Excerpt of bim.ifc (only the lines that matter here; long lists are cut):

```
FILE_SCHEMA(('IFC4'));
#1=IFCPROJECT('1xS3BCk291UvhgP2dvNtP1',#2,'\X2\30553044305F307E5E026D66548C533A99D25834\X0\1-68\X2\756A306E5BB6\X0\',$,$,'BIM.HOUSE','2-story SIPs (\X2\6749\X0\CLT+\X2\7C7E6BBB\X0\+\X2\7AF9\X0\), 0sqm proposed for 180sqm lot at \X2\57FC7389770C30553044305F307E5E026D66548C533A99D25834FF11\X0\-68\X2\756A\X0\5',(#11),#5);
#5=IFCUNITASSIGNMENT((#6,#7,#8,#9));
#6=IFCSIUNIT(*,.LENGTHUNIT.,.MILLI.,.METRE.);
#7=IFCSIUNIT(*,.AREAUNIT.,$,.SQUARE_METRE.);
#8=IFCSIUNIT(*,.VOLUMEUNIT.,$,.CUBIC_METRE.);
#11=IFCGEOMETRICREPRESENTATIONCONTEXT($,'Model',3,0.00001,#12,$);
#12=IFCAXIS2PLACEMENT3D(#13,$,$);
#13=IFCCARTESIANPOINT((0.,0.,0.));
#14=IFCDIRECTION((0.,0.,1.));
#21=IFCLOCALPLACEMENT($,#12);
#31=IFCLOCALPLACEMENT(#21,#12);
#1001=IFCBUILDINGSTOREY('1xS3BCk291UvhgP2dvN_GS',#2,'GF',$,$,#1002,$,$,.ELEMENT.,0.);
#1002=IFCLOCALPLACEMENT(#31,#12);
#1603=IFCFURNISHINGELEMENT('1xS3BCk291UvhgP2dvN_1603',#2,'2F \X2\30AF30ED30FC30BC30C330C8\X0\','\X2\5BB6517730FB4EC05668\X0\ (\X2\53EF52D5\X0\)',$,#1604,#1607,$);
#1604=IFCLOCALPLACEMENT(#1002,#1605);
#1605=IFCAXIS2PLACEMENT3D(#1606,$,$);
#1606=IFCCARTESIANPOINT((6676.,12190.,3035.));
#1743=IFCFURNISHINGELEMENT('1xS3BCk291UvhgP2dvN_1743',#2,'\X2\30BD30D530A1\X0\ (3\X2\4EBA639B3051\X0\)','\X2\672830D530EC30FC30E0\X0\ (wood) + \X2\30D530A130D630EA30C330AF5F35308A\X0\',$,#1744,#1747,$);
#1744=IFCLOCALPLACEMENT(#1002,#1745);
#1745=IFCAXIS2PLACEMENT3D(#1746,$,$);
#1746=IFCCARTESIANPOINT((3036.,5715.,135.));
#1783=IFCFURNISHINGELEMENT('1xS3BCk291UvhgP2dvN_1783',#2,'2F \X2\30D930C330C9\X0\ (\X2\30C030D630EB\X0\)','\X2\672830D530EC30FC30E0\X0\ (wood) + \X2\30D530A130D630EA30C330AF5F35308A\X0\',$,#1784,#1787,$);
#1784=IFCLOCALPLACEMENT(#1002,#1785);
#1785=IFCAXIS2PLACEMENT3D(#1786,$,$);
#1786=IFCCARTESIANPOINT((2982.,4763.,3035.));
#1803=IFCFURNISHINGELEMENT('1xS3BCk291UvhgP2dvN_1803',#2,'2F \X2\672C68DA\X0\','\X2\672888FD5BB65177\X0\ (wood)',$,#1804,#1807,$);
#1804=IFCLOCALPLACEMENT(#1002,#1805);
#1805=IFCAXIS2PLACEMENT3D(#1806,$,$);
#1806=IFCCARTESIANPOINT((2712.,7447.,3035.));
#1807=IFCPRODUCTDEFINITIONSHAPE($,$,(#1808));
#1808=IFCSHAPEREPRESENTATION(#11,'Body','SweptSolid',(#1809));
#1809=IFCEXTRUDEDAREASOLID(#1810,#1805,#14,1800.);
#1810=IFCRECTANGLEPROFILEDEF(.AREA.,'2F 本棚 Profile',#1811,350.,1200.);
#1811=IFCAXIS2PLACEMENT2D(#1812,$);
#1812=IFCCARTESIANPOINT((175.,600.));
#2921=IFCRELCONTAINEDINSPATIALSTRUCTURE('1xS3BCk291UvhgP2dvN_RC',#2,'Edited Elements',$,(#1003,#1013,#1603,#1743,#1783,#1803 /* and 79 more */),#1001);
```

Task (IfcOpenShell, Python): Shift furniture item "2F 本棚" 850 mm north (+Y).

```python
import ifcopenshell
import ifcopenshell.api.geometry
import ifcopenshell.util.placement
import ifcopenshell.util.unit

model = ifcopenshell.open("bim.ifc")
unit_scale = ifcopenshell.util.unit.calculate_unit_scale(model)

item = model.by_guid("1xS3BCk291UvhgP2dvN_1803")
matrix = ifcopenshell.util.placement.get_local_placement(item.ObjectPlacement)
matrix[1, 3] += 0.85 / unit_scale
ifcopenshell.api.geometry.edit_object_placement(model, product=item, matrix=matrix, is_si=False)

print(ifcopenshell.util.placement.get_local_placement(item.ObjectPlacement).round(3) + 0.0)

model.write("bim_rev.ifc")
```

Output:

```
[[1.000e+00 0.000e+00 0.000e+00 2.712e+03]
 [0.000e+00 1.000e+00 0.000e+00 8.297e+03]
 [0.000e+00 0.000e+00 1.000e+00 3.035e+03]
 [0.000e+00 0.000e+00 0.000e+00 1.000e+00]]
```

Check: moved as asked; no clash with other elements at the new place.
